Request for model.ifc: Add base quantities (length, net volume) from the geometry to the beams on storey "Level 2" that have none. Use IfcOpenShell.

First a look at what the model holds.

```python
import ifcopenshell
import ifcopenshell.util.element
import ifcopenshell.util.unit

model = ifcopenshell.open("model.ifc")
print(model.schema)
for unit_type in ("LENGTHUNIT", "AREAUNIT", "VOLUMEUNIT"):
    print(unit_type, ifcopenshell.util.unit.calculate_unit_scale(model, unit_type))
storey = next(s for s in model.by_type("IfcBuildingStorey") if s.Name == "Level 2")
beams = [e for e in ifcopenshell.util.element.get_decomposition(storey) if e.is_a("IfcBeam")]
for e in sorted(beams, key=lambda e: e.id()):
    print(e.id(), e.is_a(), e.Name, list(ifcopenshell.util.element.get_psets(e, qtos_only=True)), sep=" | ")
```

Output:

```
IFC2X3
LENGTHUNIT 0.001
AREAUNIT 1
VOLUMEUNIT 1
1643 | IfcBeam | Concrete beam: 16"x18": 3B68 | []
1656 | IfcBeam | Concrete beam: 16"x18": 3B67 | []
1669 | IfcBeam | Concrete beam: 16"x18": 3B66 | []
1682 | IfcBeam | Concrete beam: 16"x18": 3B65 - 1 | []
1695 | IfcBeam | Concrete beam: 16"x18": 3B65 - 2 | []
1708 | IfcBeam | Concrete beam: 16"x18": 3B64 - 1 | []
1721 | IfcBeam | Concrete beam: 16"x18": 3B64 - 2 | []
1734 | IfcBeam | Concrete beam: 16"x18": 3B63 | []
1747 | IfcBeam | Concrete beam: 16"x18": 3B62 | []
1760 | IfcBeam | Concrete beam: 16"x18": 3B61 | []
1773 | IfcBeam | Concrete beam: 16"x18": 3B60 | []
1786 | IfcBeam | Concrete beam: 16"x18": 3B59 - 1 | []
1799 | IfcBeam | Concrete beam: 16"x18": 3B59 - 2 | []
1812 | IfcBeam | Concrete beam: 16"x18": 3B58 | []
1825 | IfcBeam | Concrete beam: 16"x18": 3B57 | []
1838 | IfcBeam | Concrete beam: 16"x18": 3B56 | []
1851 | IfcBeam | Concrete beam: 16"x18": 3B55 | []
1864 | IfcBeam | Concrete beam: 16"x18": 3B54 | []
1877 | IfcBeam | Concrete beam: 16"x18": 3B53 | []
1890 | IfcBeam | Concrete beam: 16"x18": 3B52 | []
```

```python
import ifcopenshell
import ifcopenshell.api.pset
import ifcopenshell.geom
import ifcopenshell.util.element
import ifcopenshell.util.shape
import ifcopenshell.util.unit

model = ifcopenshell.open("model.ifc")
unit_scale = ifcopenshell.util.unit.calculate_unit_scale(model)
volume_scale = ifcopenshell.util.unit.calculate_unit_scale(model, "VOLUMEUNIT")
settings = ifcopenshell.geom.settings()

storey = next(s for s in model.by_type("IfcBuildingStorey") if s.Name == "Level 2")
beams = [e for e in ifcopenshell.util.element.get_decomposition(storey) if e.is_a("IfcBeam")]

for e in sorted(beams, key=lambda e: e.id()):
    if ifcopenshell.util.element.get_psets(e, qtos_only=True, should_inherit=False):
        continue
    # Geometry comes back in metres, in the element's own axes.
    shape = ifcopenshell.geom.create_shape(settings, e)
    values = {
        "Length": ifcopenshell.util.shape.get_max_xyz(shape.geometry) / unit_scale,
        "NetVolume": ifcopenshell.util.shape.get_volume(shape.geometry) / volume_scale,
    }
    qto = ifcopenshell.api.pset.add_qto(model, product=e, name="BaseQuantities")
    ifcopenshell.api.pset.edit_qto(model, qto=qto, properties=values)
    print(e.id(), {k: round(v, 3) for k, v in values.items()})

model.write("model_rev.ifc")
```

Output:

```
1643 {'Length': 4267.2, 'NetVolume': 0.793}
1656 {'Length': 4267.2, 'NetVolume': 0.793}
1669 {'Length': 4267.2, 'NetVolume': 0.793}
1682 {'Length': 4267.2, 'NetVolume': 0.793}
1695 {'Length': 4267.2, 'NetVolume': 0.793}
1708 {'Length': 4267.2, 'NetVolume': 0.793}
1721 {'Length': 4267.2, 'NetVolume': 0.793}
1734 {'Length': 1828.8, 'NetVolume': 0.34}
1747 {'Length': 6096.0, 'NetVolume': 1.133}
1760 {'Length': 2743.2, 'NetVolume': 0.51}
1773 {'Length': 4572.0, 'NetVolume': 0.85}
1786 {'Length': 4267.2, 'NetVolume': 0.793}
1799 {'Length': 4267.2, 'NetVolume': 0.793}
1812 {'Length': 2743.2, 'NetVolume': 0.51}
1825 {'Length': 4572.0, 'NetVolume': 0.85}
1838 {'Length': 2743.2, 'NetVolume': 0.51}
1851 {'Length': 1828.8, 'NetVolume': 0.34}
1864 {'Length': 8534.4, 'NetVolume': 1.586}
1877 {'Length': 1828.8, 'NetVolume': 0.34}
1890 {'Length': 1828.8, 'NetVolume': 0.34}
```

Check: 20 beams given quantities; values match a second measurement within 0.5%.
